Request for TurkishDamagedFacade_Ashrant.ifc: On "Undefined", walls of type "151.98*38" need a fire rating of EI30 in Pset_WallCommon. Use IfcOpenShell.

First a look at what the model holds.

```python
import ifcopenshell
import ifcopenshell.util.element

model = ifcopenshell.open("TurkishDamagedFacade_Ashrant.ifc")
print(model.schema)
storey = next(s for s in model.by_type("IfcBuildingStorey") if s.Name == "Undefined")
walls = [e for e in ifcopenshell.util.element.get_decomposition(storey) if e.is_a("IfcWall")]
seen = {}
for e in walls:
    element_type = ifcopenshell.util.element.get_type(e)
    key = (element_type.Name if element_type != e and element_type else None, ifcopenshell.util.element.get_pset(e, "Pset_WallCommon", "FireRating"))
    seen[key] = seen.get(key, 0) + 1
for (name, value), count in sorted(seen.items(), key=str):
    print(count, "x", name, "|", value)
```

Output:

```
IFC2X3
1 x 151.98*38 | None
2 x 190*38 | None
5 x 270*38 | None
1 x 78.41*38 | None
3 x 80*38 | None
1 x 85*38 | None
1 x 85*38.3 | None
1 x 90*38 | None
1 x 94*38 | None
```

```python
import ifcopenshell
import ifcopenshell.api.pset
import ifcopenshell.util.element

model = ifcopenshell.open("TurkishDamagedFacade_Ashrant.ifc")

storey = next(s for s in model.by_type("IfcBuildingStorey") if s.Name == "Undefined")
walls = [e for e in ifcopenshell.util.element.get_decomposition(storey) if e.is_a("IfcWall")]

count = 0
for e in walls:
    element_type = ifcopenshell.util.element.get_type(e)
    if element_type in (None, e) or element_type.Name != "151.98*38":
        continue
    # add_pset returns the element's existing set when there is one.
    pset = ifcopenshell.api.pset.add_pset(model, product=e, name="Pset_WallCommon")
    ifcopenshell.api.pset.edit_pset(model, pset=pset, properties={"FireRating": "EI30"})
    count += 1

print(count, "walls updated")

model.write("TurkishDamagedFacade_Ashrant_edited.ifc")
```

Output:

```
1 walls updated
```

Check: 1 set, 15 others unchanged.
